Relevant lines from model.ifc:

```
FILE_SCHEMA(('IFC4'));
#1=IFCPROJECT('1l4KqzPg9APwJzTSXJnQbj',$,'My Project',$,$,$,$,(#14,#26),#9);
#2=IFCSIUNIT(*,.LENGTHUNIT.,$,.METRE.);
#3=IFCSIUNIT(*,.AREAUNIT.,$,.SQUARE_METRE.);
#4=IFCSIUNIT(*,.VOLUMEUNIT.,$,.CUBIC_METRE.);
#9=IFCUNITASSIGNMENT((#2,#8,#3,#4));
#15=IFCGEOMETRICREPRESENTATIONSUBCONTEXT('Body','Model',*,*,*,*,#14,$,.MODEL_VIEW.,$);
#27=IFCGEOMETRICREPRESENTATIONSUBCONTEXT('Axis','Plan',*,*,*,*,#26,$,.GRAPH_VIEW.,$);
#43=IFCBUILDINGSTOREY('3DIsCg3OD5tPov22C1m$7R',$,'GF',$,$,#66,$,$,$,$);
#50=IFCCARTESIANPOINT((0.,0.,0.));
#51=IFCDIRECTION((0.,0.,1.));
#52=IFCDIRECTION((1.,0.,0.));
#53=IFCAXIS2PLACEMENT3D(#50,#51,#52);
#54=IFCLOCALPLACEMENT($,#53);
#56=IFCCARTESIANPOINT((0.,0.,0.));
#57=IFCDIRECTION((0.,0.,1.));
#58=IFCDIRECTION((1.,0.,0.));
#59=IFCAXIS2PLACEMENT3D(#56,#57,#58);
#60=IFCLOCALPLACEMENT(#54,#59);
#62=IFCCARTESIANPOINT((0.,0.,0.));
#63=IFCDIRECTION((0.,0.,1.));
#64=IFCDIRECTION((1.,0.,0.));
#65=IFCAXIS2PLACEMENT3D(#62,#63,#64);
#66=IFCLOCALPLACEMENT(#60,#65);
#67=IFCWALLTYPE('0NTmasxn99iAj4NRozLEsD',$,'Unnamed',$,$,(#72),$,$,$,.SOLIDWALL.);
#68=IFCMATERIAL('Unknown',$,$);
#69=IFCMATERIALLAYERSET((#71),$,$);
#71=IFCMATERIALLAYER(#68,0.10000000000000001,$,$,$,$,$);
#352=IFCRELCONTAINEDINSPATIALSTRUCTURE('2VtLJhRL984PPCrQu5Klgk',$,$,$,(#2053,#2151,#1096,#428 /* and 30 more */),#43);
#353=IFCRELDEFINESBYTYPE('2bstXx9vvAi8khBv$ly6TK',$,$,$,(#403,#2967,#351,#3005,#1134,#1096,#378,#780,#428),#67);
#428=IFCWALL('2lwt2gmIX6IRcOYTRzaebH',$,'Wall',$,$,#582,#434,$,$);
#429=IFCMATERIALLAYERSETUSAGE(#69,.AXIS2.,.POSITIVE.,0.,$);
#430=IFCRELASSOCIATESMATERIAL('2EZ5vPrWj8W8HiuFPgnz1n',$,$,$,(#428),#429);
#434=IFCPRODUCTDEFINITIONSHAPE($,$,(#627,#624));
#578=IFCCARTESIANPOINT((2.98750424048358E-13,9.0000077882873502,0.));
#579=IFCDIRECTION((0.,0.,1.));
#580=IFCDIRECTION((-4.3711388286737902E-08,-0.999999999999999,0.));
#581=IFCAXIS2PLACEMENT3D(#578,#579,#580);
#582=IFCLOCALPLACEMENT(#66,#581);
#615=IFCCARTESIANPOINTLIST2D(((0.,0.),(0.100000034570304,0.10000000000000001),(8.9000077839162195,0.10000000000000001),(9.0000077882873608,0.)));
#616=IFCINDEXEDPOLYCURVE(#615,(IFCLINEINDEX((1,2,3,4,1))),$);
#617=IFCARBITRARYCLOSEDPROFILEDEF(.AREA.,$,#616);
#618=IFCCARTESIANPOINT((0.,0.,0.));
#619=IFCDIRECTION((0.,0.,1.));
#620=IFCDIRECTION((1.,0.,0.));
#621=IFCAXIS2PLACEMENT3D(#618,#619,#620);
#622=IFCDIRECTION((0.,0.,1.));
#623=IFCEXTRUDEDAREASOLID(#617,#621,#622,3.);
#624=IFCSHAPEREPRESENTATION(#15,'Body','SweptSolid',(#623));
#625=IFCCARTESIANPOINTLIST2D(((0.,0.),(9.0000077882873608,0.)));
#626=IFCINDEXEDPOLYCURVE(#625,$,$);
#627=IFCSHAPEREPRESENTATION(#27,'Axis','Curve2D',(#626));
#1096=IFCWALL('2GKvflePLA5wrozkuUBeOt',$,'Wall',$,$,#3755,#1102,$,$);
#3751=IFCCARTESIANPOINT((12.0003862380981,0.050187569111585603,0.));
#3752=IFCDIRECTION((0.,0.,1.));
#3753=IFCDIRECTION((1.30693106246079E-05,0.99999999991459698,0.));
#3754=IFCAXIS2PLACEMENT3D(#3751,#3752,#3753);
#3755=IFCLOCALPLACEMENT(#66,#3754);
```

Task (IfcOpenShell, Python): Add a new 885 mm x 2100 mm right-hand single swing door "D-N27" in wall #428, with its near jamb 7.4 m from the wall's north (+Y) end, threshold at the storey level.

```python
import numpy as np
import ifcopenshell
import ifcopenshell.api.feature
import ifcopenshell.api.geometry
import ifcopenshell.api.root
import ifcopenshell.api.spatial
import ifcopenshell.geom
import ifcopenshell.util.element
import ifcopenshell.util.placement
import ifcopenshell.util.representation
import ifcopenshell.util.shape
import ifcopenshell.util.unit

model = ifcopenshell.open("model.ifc")
unit_scale = ifcopenshell.util.unit.calculate_unit_scale(model)
settings = ifcopenshell.geom.settings()


def volume(element):
    """Net volume in cubic metres, openings subtracted."""
    shape = ifcopenshell.geom.create_shape(settings, element)
    return ifcopenshell.util.shape.get_volume(shape.geometry)


wall = model.by_guid("2lwt2gmIX6IRcOYTRzaebH")
storey = ifcopenshell.util.element.get_container(wall, ifc_class="IfcBuildingStorey")
context = ifcopenshell.util.representation.get_context(model, "Model", "Body", "MODEL_VIEW")
before = volume(wall)

width, height, from_end, sill = 0.885, 2.1, 7.4, 0.0  # metres

# The wall runs along its own X axis, and the end named is its -X end.
wall_shape = ifcopenshell.geom.create_shape(settings, wall)
x, y, z = ifcopenshell.util.shape.get_vertices(wall_shape.geometry).T
start = x.min() + from_end
face, thickness = float(y.min()), float(y.max() - y.min())
wall_matrix = ifcopenshell.util.placement.get_local_placement(wall.ObjectPlacement)
level = ifcopenshell.util.placement.get_local_placement(storey.ObjectPlacement)[2, 3]


def in_wall(x, y):
    """Placement at x, y metres in the wall's axes, at sill height."""
    matrix = wall_matrix.copy()
    matrix[:, 3] = wall_matrix @ np.array([x / unit_scale, y / unit_scale, 0.0, 1.0])
    matrix[2, 3] = level + sill / unit_scale
    return matrix


# Opening: a box that overshoots both wall faces by 50 mm.
opening = ifcopenshell.api.root.create_entity(model, ifc_class="IfcOpeningElement", predefined_type="OPENING")
box = ifcopenshell.api.geometry.add_wall_representation(
    model, context=context, length=width, height=height, thickness=thickness + 0.1
)
ifcopenshell.api.geometry.assign_representation(model, product=opening, representation=box)
ifcopenshell.api.geometry.edit_object_placement(model, product=opening, matrix=in_wall(start, face - 0.05), is_si=False)
ifcopenshell.api.feature.add_feature(model, feature=opening, element=wall)

door = ifcopenshell.api.root.create_entity(model, ifc_class="IfcDoor", name="D-N27", predefined_type="DOOR")
door.OverallWidth, door.OverallHeight = width / unit_scale, height / unit_scale
door.OperationType = "SINGLE_SWING_RIGHT"
body = ifcopenshell.api.geometry.add_door_representation(
    model,
    context=context,
    overall_width=door.OverallWidth,
    overall_height=door.OverallHeight,
    operation_type="SINGLE_SWING_RIGHT",
    lining_properties={"LiningDepth": thickness / unit_scale, "ThresholdDepth": thickness / unit_scale},
)
ifcopenshell.api.geometry.assign_representation(model, product=door, representation=body)
ifcopenshell.api.spatial.assign_container(model, products=[door], relating_structure=storey)
ifcopenshell.api.feature.add_filling(model, opening=opening, element=door)

# The lining spans the wall, so the door starts at the wall face.
ifcopenshell.api.geometry.edit_object_placement(model, product=door, matrix=in_wall(start, face), is_si=False)

after = volume(wall)

print(f"wall volume {before:.3f} -> {after:.3f} m3")

model.write("model-out.ifc")
```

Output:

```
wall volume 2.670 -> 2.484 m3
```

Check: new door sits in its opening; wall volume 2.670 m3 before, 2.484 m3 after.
